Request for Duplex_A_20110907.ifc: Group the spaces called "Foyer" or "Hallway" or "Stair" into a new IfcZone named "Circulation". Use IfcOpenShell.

First a look at what the model holds.

```python
import ifcopenshell

model = ifcopenshell.open("Duplex_A_20110907.ifc")
print(model.schema)
seen = {}
for space in model.by_type("IfcSpace"):
    seen[space.LongName] = seen.get(space.LongName, 0) + 1
for name, count in sorted(seen.items(), key=str):
    print(count, "x", name)
print("zones:", [z.Name for z in model.by_type("IfcZone")][:20])
```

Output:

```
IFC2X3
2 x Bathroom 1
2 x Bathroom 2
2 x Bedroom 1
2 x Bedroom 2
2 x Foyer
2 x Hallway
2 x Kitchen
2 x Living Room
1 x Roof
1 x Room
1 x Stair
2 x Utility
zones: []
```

```python
import ifcopenshell
import ifcopenshell.api.group
import ifcopenshell.api.root

model = ifcopenshell.open("Duplex_A_20110907.ifc")

names = {"Foyer", "Hallway", "Stair"}
spaces = [s for s in model.by_type("IfcSpace") if s.LongName in names]

zone = ifcopenshell.api.root.create_entity(model, ifc_class="IfcZone", name="Circulation")
ifcopenshell.api.group.assign_group(model, products=spaces, group=zone)
print(len(spaces), "spaces in", zone.Name)

model.write("Duplex_A_20110907_v2.ifc")
```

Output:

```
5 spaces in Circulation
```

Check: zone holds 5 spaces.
